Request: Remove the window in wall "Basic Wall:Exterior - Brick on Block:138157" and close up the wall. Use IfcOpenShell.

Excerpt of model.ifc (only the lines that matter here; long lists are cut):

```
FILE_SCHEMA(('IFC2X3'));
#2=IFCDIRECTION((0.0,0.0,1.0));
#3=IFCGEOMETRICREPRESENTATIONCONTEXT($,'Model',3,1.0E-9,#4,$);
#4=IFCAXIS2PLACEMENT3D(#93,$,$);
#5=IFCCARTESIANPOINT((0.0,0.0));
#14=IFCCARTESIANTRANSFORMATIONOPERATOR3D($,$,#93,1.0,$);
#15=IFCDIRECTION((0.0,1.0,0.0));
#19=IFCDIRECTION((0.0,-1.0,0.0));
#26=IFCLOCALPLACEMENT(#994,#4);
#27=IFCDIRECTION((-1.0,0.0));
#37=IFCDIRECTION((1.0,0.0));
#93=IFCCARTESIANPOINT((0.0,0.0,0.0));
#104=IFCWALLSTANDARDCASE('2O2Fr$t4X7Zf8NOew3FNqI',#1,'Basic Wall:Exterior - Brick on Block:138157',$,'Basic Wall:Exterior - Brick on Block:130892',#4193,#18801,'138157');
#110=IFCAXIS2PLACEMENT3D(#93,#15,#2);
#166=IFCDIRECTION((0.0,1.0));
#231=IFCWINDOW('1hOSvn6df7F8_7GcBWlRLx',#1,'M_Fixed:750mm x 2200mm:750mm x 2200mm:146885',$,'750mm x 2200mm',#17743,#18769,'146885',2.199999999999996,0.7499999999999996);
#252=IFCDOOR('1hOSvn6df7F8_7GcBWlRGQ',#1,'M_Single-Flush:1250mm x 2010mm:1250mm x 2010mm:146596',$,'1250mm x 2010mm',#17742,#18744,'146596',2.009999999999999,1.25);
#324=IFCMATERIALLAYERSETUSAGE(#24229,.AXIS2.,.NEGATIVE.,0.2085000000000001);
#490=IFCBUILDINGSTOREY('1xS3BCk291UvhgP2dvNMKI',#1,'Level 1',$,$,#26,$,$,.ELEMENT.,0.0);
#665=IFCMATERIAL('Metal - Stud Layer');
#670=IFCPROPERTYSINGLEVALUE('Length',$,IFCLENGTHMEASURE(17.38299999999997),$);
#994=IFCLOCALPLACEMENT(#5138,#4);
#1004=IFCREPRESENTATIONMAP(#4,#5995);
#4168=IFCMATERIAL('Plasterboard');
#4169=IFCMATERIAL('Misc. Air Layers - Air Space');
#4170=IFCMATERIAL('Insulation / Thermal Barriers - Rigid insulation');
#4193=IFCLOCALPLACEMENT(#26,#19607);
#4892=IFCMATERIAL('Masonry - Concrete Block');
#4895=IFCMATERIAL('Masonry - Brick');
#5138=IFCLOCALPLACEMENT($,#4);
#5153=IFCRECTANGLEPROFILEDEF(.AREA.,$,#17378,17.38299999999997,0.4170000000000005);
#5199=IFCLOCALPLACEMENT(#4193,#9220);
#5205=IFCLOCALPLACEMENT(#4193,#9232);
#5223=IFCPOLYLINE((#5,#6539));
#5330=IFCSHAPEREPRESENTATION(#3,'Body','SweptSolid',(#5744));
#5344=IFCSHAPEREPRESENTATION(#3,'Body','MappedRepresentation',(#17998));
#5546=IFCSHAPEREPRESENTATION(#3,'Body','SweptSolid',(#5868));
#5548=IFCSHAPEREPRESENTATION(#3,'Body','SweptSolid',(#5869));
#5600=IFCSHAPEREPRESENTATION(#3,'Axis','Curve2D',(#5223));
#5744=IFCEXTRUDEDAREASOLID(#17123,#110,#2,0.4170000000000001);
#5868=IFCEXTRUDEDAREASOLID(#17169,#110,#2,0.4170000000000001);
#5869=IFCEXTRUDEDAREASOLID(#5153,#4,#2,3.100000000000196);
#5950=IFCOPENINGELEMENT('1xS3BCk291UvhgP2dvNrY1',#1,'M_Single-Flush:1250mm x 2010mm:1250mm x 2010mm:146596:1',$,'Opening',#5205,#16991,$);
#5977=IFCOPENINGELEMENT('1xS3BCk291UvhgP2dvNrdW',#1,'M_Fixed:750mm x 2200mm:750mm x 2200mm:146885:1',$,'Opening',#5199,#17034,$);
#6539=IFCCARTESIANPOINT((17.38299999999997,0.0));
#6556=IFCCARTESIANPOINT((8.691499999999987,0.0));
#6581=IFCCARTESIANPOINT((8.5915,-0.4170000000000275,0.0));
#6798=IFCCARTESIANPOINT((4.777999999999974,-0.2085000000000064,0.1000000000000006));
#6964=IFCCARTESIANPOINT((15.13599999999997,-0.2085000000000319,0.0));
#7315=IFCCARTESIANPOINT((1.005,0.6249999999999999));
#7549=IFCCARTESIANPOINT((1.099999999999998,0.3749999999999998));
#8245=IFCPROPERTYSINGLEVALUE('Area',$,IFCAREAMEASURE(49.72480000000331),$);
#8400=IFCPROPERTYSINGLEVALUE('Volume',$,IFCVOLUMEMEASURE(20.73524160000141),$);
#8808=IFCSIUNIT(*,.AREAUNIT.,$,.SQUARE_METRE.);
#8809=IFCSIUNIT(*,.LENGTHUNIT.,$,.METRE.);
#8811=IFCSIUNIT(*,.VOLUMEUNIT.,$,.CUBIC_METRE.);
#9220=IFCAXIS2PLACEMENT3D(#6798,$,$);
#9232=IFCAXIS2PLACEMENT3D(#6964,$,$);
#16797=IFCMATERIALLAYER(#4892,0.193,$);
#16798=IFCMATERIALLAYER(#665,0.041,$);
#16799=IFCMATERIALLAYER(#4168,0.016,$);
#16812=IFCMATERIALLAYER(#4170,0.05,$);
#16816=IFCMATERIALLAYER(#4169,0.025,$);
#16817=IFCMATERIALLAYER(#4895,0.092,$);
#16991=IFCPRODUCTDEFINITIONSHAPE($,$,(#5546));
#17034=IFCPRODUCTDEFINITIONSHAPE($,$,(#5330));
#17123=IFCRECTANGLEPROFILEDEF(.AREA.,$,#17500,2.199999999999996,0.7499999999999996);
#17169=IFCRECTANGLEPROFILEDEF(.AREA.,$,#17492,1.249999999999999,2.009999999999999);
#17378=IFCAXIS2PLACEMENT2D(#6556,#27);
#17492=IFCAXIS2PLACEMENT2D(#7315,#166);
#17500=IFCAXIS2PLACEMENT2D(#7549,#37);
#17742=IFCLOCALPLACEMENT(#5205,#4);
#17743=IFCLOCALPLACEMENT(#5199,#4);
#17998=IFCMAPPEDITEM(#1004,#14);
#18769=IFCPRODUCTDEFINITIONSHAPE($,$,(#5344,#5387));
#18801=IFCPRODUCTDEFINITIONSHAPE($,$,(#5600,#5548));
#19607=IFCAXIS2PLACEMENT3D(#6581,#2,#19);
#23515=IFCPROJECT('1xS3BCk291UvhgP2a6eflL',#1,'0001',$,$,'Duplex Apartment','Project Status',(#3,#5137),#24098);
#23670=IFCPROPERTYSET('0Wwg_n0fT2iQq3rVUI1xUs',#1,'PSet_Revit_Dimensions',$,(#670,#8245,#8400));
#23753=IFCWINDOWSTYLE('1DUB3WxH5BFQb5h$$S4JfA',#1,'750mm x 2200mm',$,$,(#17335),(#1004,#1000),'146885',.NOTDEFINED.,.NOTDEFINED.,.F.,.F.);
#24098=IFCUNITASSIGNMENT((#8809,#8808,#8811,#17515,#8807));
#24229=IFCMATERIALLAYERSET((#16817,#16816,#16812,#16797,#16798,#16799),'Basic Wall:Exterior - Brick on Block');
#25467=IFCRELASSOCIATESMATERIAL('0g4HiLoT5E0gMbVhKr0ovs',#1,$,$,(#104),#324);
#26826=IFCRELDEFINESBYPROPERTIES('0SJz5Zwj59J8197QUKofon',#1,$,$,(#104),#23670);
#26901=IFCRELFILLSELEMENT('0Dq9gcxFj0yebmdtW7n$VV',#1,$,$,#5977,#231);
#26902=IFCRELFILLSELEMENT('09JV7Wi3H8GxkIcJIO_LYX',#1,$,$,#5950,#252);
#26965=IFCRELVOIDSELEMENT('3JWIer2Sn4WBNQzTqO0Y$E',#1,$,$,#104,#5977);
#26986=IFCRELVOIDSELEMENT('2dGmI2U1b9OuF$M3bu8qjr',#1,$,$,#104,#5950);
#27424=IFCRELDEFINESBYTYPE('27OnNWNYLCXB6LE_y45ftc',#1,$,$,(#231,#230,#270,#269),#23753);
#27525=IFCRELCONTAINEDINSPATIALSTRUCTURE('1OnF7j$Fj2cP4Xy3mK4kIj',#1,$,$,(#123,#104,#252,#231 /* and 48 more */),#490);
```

```python
import ifcopenshell
import ifcopenshell.api.feature
import ifcopenshell.api.pset
import ifcopenshell.api.root
import ifcopenshell.geom
import ifcopenshell.util.element
import ifcopenshell.util.shape
import ifcopenshell.util.unit

model = ifcopenshell.open("model.ifc")
area_scale = ifcopenshell.util.unit.calculate_unit_scale(model, "AREAUNIT")
volume_scale = ifcopenshell.util.unit.calculate_unit_scale(model, "VOLUMEUNIT")
settings = ifcopenshell.geom.settings()


def volume(element):
    """Net volume in cubic metres, openings subtracted."""
    shape = ifcopenshell.geom.create_shape(settings, element)
    return ifcopenshell.util.shape.get_volume(shape.geometry)


window = model.by_guid("1hOSvn6df7F8_7GcBWlRLx")
opening = window.FillsVoids[0].RelatingOpeningElement
wall = opening.VoidsElements[0].RelatingBuildingElement
before = volume(wall)

ifcopenshell.api.root.remove_product(model, product=window)
ifcopenshell.api.feature.remove_feature(model, feature=opening)

after = volume(wall)
thickness = 0.417  # wall thickness in metres

# Update the wall's stored quantities.
pset = model.by_id(ifcopenshell.util.element.get_pset(wall, "PSet_Revit_Dimensions", should_inherit=False)["id"])
ifcopenshell.api.pset.edit_pset(model, pset=pset, properties={
    "Area": model.create_entity("IfcAreaMeasure", after / thickness / area_scale),
    "Volume": model.create_entity("IfcVolumeMeasure", after / volume_scale),
})

print(f"wall volume {before:.3f} -> {after:.3f} m3")

model.write("model_updated.ifc")
```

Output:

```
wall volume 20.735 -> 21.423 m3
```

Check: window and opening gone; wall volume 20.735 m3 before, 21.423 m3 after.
